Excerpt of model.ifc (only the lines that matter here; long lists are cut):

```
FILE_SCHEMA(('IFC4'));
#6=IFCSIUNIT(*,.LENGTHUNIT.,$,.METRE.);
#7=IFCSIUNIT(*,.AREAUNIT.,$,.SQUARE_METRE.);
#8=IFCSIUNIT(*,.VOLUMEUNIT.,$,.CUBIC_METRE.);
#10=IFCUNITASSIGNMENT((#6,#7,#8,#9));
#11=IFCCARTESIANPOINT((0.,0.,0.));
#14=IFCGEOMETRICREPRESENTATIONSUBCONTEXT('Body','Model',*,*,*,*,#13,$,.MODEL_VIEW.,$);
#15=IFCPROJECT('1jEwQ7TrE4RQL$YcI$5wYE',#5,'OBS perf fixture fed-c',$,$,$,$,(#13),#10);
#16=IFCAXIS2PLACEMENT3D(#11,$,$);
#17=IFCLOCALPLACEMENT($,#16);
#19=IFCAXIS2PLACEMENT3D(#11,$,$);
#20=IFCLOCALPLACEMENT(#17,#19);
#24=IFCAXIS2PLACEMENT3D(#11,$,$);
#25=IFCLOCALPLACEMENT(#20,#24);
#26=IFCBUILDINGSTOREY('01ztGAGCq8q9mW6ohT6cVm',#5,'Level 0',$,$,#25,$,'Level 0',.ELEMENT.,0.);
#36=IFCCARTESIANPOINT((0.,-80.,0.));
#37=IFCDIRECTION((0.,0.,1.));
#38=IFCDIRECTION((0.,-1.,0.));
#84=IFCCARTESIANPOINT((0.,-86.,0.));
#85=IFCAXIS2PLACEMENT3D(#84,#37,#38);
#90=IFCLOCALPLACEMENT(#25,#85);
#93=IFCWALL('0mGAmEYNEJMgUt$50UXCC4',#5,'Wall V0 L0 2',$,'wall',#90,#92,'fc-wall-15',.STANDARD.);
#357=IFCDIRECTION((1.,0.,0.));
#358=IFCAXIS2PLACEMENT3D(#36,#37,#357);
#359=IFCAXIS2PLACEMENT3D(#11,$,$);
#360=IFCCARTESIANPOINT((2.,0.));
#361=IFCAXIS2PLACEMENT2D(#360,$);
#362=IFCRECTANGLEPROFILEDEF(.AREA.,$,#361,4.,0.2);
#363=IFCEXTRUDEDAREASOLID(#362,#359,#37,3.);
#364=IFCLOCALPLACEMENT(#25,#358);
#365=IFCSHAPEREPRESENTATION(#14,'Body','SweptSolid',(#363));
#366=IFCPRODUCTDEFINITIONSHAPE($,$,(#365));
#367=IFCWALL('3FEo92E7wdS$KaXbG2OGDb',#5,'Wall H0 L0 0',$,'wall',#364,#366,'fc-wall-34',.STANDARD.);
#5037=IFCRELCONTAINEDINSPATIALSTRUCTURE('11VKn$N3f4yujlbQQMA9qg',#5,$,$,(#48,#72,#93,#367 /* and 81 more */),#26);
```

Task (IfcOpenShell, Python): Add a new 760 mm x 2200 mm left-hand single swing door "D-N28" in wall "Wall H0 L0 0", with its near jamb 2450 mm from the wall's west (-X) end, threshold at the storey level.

```python
import numpy as np
import ifcopenshell
import ifcopenshell.api.feature
import ifcopenshell.api.geometry
import ifcopenshell.api.root
import ifcopenshell.api.spatial
import ifcopenshell.geom
import ifcopenshell.util.element
import ifcopenshell.util.placement
import ifcopenshell.util.representation
import ifcopenshell.util.shape
import ifcopenshell.util.unit

model = ifcopenshell.open("model.ifc")
unit_scale = ifcopenshell.util.unit.calculate_unit_scale(model)
settings = ifcopenshell.geom.settings()


def volume(element):
    """Net volume in cubic metres, openings subtracted."""
    shape = ifcopenshell.geom.create_shape(settings, element)
    return ifcopenshell.util.shape.get_volume(shape.geometry)


wall = model.by_guid("3FEo92E7wdS$KaXbG2OGDb")
storey = ifcopenshell.util.element.get_container(wall, ifc_class="IfcBuildingStorey")
context = ifcopenshell.util.representation.get_context(model, "Model", "Body", "MODEL_VIEW")
before = volume(wall)

width, height, from_end, sill = 0.76, 2.2, 2.45, 0.0  # metres

# The wall runs along its own X axis, and the end named is its -X end.
wall_shape = ifcopenshell.geom.create_shape(settings, wall)
x, y, z = ifcopenshell.util.shape.get_vertices(wall_shape.geometry).T
start = x.min() + from_end
face, thickness = float(y.min()), float(y.max() - y.min())
wall_matrix = ifcopenshell.util.placement.get_local_placement(wall.ObjectPlacement)
level = ifcopenshell.util.placement.get_local_placement(storey.ObjectPlacement)[2, 3]


def in_wall(x, y):
    """Placement at x, y metres in the wall's axes, at sill height."""
    matrix = wall_matrix.copy()
    matrix[:, 3] = wall_matrix @ np.array([x / unit_scale, y / unit_scale, 0.0, 1.0])
    matrix[2, 3] = level + sill / unit_scale
    return matrix


# Opening: a box that overshoots both wall faces by 50 mm.
opening = ifcopenshell.api.root.create_entity(model, ifc_class="IfcOpeningElement", predefined_type="OPENING")
box = ifcopenshell.api.geometry.add_wall_representation(
    model, context=context, length=width, height=height, thickness=thickness + 0.1
)
ifcopenshell.api.geometry.assign_representation(model, product=opening, representation=box)
ifcopenshell.api.geometry.edit_object_placement(model, product=opening, matrix=in_wall(start, face - 0.05), is_si=False)
ifcopenshell.api.feature.add_feature(model, feature=opening, element=wall)

door = ifcopenshell.api.root.create_entity(model, ifc_class="IfcDoor", name="D-N28", predefined_type="DOOR")
door.OverallWidth, door.OverallHeight = width / unit_scale, height / unit_scale
door.OperationType = "SINGLE_SWING_LEFT"
body = ifcopenshell.api.geometry.add_door_representation(
    model,
    context=context,
    overall_width=door.OverallWidth,
    overall_height=door.OverallHeight,
    operation_type="SINGLE_SWING_LEFT",
    lining_properties={"LiningDepth": thickness / unit_scale, "ThresholdDepth": thickness / unit_scale},
)
ifcopenshell.api.geometry.assign_representation(model, product=door, representation=body)
ifcopenshell.api.spatial.assign_container(model, products=[door], relating_structure=storey)
ifcopenshell.api.feature.add_filling(model, opening=opening, element=door)

# The lining spans the wall, so the door starts at the wall face.
ifcopenshell.api.geometry.edit_object_placement(model, product=door, matrix=in_wall(start, face), is_si=False)

after = volume(wall)

print(f"wall volume {before:.3f} -> {after:.3f} m3")

model.write("model_v2.ifc")
```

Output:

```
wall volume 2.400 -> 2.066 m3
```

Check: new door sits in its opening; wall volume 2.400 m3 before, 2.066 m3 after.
